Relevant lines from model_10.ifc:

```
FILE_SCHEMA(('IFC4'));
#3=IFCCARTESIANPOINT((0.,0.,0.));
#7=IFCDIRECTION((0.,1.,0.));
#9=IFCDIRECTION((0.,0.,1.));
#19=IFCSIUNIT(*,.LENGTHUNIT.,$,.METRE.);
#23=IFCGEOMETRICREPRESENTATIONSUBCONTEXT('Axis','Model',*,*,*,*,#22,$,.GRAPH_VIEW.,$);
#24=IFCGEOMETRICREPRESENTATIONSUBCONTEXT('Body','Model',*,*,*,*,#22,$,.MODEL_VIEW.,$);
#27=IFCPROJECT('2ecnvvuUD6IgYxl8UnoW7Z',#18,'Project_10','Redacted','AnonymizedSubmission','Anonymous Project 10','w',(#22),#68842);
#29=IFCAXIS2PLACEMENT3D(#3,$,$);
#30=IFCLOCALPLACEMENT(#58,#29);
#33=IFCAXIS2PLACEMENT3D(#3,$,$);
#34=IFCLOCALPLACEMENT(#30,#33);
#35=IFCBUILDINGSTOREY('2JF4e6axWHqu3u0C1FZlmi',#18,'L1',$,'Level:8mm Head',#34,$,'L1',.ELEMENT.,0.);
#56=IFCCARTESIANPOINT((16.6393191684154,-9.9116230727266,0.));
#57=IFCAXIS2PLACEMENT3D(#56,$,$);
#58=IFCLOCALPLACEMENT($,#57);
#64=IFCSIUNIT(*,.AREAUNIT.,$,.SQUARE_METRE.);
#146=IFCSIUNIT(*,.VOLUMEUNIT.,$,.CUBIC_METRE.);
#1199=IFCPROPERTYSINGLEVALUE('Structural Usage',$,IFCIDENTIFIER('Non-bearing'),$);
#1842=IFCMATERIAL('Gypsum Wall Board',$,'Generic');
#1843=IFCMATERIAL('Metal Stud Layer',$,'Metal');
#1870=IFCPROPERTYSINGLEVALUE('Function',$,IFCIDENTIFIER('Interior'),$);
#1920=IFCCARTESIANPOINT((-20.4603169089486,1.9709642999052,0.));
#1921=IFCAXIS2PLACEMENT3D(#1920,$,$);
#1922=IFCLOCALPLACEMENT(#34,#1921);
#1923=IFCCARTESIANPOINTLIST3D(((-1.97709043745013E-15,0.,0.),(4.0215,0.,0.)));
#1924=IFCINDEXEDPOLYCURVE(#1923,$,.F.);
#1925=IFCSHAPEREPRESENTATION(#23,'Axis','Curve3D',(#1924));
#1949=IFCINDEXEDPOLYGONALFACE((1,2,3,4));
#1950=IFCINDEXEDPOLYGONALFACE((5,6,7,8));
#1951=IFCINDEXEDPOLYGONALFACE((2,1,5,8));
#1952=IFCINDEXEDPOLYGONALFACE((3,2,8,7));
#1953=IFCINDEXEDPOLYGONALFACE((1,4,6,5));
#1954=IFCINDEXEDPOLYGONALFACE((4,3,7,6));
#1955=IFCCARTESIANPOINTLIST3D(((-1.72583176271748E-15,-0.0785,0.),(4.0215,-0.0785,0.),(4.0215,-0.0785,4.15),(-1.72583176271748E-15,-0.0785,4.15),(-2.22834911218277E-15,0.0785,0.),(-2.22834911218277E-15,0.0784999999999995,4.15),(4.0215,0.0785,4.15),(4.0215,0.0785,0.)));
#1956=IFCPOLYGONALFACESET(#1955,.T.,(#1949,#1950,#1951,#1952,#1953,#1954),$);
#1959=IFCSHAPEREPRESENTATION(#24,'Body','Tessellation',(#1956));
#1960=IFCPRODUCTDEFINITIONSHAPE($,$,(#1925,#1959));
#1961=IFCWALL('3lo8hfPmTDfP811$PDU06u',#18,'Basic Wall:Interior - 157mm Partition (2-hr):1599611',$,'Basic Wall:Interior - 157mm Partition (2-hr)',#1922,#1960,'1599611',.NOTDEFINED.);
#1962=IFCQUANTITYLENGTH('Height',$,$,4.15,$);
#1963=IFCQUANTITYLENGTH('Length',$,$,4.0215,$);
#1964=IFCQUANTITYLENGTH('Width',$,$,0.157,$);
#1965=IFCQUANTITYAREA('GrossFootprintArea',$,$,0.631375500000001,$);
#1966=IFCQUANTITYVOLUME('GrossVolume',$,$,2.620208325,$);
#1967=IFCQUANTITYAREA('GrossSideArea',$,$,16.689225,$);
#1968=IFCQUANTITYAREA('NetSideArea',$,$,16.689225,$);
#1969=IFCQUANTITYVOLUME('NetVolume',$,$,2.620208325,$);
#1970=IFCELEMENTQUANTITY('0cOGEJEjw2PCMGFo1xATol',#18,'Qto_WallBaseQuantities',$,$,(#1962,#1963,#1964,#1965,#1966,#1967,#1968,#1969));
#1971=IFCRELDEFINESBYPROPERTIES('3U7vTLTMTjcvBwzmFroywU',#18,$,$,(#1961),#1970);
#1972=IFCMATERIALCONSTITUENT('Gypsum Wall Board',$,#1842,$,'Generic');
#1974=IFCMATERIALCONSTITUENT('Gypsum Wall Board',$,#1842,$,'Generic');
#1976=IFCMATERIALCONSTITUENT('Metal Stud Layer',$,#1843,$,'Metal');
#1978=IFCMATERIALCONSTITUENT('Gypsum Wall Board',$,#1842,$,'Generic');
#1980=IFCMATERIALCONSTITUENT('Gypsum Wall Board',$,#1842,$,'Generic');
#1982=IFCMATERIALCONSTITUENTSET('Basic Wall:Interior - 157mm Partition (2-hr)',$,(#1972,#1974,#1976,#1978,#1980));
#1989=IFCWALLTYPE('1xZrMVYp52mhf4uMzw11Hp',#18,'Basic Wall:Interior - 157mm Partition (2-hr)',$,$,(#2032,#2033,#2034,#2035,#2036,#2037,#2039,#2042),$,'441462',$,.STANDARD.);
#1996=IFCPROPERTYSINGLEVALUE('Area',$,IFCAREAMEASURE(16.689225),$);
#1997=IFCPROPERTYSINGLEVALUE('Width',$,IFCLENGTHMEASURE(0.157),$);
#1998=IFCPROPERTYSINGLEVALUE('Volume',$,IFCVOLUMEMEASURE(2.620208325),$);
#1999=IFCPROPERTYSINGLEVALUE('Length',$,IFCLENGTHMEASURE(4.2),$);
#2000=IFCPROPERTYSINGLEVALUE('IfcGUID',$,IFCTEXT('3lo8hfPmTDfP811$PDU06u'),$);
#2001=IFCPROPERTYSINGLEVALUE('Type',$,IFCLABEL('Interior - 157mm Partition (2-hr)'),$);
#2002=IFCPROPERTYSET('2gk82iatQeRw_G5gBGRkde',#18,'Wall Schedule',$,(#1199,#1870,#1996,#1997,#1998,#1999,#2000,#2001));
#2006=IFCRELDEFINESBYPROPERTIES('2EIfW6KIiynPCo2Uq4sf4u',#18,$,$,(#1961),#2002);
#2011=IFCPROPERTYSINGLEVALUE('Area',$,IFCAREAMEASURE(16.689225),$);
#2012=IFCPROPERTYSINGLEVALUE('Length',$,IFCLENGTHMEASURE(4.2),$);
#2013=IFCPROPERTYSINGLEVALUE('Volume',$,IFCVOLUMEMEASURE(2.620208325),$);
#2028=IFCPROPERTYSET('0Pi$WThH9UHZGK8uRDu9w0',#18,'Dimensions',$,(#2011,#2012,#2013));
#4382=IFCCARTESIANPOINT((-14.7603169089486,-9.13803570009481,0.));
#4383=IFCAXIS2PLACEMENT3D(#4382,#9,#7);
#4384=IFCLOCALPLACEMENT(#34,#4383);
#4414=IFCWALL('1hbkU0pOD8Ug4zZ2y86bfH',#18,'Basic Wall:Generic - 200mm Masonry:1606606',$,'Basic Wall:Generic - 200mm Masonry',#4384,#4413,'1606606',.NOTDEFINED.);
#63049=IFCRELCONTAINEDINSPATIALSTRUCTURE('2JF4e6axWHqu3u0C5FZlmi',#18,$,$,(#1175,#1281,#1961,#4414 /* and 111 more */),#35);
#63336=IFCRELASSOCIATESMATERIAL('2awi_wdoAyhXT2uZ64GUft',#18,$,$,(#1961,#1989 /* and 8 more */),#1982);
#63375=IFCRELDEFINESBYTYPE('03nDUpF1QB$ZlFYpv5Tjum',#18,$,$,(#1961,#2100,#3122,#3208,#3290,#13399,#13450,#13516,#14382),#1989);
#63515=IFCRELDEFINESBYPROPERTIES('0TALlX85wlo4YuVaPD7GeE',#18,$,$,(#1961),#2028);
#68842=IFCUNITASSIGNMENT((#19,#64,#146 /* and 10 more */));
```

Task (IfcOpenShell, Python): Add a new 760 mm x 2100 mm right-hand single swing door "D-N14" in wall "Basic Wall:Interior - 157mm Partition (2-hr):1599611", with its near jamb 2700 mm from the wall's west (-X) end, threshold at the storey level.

```python
import numpy as np
import ifcopenshell
import ifcopenshell.api.feature
import ifcopenshell.api.geometry
import ifcopenshell.api.pset
import ifcopenshell.api.root
import ifcopenshell.api.spatial
import ifcopenshell.geom
import ifcopenshell.util.element
import ifcopenshell.util.placement
import ifcopenshell.util.representation
import ifcopenshell.util.shape
import ifcopenshell.util.unit

model = ifcopenshell.open("model_10.ifc")
unit_scale = ifcopenshell.util.unit.calculate_unit_scale(model)
area_scale = ifcopenshell.util.unit.calculate_unit_scale(model, "AREAUNIT")
volume_scale = ifcopenshell.util.unit.calculate_unit_scale(model, "VOLUMEUNIT")
settings = ifcopenshell.geom.settings()


def volume(element):
    """Net volume in cubic metres, openings subtracted."""
    shape = ifcopenshell.geom.create_shape(settings, element)
    return ifcopenshell.util.shape.get_volume(shape.geometry)


wall = model.by_guid("3lo8hfPmTDfP811$PDU06u")
storey = ifcopenshell.util.element.get_container(wall, ifc_class="IfcBuildingStorey")
context = ifcopenshell.util.representation.get_context(model, "Model", "Body", "MODEL_VIEW")
before = volume(wall)

width, height, from_end, sill = 0.76, 2.1, 2.7, 0.0  # metres

# The wall runs along its own X axis, and the end named is its -X end.
wall_shape = ifcopenshell.geom.create_shape(settings, wall)
x, y, z = ifcopenshell.util.shape.get_vertices(wall_shape.geometry).T
start = x.min() + from_end
face, thickness = float(y.min()), float(y.max() - y.min())
wall_matrix = ifcopenshell.util.placement.get_local_placement(wall.ObjectPlacement)
level = ifcopenshell.util.placement.get_local_placement(storey.ObjectPlacement)[2, 3]


def in_wall(x, y):
    """Placement at x, y metres in the wall's axes, at sill height."""
    matrix = wall_matrix.copy()
    matrix[:, 3] = wall_matrix @ np.array([x / unit_scale, y / unit_scale, 0.0, 1.0])
    matrix[2, 3] = level + sill / unit_scale
    return matrix


# Opening: a box that overshoots both wall faces by 50 mm.
opening = ifcopenshell.api.root.create_entity(model, ifc_class="IfcOpeningElement", predefined_type="OPENING")
box = ifcopenshell.api.geometry.add_wall_representation(
    model, context=context, length=width, height=height, thickness=thickness + 0.1
)
ifcopenshell.api.geometry.assign_representation(model, product=opening, representation=box)
ifcopenshell.api.geometry.edit_object_placement(model, product=opening, matrix=in_wall(start, face - 0.05), is_si=False)
ifcopenshell.api.feature.add_feature(model, feature=opening, element=wall)

door = ifcopenshell.api.root.create_entity(model, ifc_class="IfcDoor", name="D-N14", predefined_type="DOOR")
door.OverallWidth, door.OverallHeight = width / unit_scale, height / unit_scale
door.OperationType = "SINGLE_SWING_RIGHT"
body = ifcopenshell.api.geometry.add_door_representation(
    model,
    context=context,
    overall_width=door.OverallWidth,
    overall_height=door.OverallHeight,
    operation_type="SINGLE_SWING_RIGHT",
    lining_properties={"LiningDepth": thickness / unit_scale, "ThresholdDepth": thickness / unit_scale},
)
ifcopenshell.api.geometry.assign_representation(model, product=door, representation=body)
ifcopenshell.api.spatial.assign_container(model, products=[door], relating_structure=storey)
ifcopenshell.api.feature.add_filling(model, opening=opening, element=door)

# The lining spans the wall, so the door starts at the wall face.
ifcopenshell.api.geometry.edit_object_placement(model, product=door, matrix=in_wall(start, face), is_si=False)

after = volume(wall)

# Update the wall's stored quantities.
qto = model.by_id(ifcopenshell.util.element.get_pset(wall, "Qto_WallBaseQuantities", should_inherit=False)["id"])
ifcopenshell.api.pset.edit_qto(model, qto=qto, properties={
    "NetSideArea": after / thickness / area_scale,
    "NetVolume": after / volume_scale,
})
pset = model.by_id(ifcopenshell.util.element.get_pset(wall, "Wall Schedule", should_inherit=False)["id"])
ifcopenshell.api.pset.edit_pset(model, pset=pset, properties={
    "Area": model.create_entity("IfcAreaMeasure", after / thickness / area_scale),
    "Volume": model.create_entity("IfcVolumeMeasure", after / volume_scale),
})
pset = model.by_id(ifcopenshell.util.element.get_pset(wall, "Dimensions", should_inherit=False)["id"])
ifcopenshell.api.pset.edit_pset(model, pset=pset, properties={
    "Area": model.create_entity("IfcAreaMeasure", after / thickness / area_scale),
    "Volume": model.create_entity("IfcVolumeMeasure", after / volume_scale),
})

print(f"wall volume {before:.3f} -> {after:.3f} m3")

model.write("model_10-out.ifc")
```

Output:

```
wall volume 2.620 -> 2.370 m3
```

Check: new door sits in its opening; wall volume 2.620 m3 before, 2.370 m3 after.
